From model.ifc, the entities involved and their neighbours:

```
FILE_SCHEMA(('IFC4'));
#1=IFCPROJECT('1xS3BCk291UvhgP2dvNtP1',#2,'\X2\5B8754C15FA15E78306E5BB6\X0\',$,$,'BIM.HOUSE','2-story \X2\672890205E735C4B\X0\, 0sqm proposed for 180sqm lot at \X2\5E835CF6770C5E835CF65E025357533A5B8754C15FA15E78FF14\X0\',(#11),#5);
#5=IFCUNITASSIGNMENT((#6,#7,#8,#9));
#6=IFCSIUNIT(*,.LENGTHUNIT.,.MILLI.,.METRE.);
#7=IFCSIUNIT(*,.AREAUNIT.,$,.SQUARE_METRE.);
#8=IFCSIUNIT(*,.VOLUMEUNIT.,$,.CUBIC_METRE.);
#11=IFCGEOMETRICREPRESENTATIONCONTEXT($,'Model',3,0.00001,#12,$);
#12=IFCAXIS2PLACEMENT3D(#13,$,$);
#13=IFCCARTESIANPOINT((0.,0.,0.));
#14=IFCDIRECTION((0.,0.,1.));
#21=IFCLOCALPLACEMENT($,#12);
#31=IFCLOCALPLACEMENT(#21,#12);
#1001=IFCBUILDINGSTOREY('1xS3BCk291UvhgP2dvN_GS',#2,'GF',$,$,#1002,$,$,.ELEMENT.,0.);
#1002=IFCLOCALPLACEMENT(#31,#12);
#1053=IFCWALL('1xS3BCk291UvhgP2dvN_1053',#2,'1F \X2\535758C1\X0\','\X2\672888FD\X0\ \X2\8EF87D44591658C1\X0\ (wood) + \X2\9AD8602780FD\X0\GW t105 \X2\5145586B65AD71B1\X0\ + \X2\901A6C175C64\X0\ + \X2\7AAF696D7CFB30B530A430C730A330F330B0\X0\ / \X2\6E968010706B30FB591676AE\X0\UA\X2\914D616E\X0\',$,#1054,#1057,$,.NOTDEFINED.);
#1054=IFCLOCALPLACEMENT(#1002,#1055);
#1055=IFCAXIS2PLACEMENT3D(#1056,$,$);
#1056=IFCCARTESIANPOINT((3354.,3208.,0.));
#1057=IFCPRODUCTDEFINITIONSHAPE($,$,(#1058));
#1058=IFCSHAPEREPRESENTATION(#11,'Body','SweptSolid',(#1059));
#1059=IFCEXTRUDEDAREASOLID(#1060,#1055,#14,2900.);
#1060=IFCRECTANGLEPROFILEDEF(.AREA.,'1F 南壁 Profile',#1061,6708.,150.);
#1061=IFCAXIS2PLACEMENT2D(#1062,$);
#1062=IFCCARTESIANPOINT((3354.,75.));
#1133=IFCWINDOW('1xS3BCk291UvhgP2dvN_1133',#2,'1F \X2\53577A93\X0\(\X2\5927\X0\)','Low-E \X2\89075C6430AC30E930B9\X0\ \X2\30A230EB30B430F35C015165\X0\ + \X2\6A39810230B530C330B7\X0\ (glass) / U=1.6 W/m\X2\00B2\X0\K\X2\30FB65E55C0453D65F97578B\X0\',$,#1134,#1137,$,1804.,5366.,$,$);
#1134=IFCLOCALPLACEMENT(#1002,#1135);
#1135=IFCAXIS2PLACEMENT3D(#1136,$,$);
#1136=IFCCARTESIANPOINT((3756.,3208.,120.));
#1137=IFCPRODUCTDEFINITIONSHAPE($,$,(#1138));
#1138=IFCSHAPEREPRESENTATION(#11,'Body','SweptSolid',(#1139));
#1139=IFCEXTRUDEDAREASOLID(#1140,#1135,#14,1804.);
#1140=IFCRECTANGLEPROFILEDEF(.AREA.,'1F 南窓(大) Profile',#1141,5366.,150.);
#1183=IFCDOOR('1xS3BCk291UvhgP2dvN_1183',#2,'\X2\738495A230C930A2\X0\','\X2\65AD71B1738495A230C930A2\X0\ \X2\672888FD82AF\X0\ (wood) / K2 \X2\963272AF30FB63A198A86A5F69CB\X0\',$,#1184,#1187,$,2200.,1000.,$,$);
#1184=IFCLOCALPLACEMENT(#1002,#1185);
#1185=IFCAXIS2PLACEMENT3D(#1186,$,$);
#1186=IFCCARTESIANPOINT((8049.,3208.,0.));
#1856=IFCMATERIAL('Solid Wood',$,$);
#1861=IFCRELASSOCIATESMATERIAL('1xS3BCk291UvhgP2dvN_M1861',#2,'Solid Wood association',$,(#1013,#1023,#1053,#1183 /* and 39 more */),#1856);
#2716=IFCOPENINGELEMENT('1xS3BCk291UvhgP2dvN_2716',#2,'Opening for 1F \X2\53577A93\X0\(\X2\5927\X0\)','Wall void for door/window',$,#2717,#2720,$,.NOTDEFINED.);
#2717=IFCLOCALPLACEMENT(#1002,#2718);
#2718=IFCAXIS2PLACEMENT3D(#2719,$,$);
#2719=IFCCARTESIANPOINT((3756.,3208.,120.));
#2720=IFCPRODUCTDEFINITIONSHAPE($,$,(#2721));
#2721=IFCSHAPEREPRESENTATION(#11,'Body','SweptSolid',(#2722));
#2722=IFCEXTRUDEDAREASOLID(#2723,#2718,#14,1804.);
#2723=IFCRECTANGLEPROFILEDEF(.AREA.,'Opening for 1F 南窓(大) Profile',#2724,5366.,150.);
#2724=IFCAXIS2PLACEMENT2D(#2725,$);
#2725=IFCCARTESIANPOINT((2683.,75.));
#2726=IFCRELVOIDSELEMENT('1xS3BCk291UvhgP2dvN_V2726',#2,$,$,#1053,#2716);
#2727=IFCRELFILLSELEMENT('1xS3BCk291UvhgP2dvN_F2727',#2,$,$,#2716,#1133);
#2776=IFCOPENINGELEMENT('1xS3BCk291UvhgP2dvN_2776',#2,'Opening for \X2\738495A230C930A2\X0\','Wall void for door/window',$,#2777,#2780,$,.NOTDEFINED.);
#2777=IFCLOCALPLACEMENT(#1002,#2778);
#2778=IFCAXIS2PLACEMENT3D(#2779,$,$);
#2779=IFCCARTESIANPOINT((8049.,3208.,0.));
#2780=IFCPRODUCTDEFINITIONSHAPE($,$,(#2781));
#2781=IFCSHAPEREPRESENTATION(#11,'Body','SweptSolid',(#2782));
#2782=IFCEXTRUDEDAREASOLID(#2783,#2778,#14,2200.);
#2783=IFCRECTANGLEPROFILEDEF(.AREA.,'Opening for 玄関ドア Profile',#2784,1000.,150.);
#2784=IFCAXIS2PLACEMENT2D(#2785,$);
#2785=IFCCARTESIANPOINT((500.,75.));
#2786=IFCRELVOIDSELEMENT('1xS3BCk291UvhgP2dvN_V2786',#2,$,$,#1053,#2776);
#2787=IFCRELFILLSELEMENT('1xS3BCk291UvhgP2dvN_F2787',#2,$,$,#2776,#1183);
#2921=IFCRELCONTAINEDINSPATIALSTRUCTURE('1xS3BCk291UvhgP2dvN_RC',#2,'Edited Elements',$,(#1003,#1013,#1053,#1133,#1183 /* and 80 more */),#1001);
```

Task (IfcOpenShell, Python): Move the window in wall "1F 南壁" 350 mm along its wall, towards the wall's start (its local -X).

```python
import ifcopenshell
import ifcopenshell.api.geometry
import ifcopenshell.util.placement
import ifcopenshell.util.unit

model = ifcopenshell.open("model.ifc")
unit_scale = ifcopenshell.util.unit.calculate_unit_scale(model)

window = model.by_guid("1xS3BCk291UvhgP2dvN_1133")
opening = window.FillsVoids[0].RelatingOpeningElement
wall = opening.VoidsElements[0].RelatingBuildingElement

wall_matrix = ifcopenshell.util.placement.get_local_placement(wall.ObjectPlacement)
shift = wall_matrix[:3, 0] * -0.35 / unit_scale
before = ifcopenshell.util.placement.get_local_placement(window.ObjectPlacement)[:3, 3].copy()

# The window is not placed relative to its opening, so move both.
for product in (opening, window):
    matrix = ifcopenshell.util.placement.get_local_placement(product.ObjectPlacement)
    matrix[:3, 3] += shift
    ifcopenshell.api.geometry.edit_object_placement(model, product=product, matrix=matrix, is_si=False)

after = ifcopenshell.util.placement.get_local_placement(window.ObjectPlacement)[:3, 3]
print("window moved by", (after - before).round(3) + 0.0)

model.write("model_updated.ifc")
```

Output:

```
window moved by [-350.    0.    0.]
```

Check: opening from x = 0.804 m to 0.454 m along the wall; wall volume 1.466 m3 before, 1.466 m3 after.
